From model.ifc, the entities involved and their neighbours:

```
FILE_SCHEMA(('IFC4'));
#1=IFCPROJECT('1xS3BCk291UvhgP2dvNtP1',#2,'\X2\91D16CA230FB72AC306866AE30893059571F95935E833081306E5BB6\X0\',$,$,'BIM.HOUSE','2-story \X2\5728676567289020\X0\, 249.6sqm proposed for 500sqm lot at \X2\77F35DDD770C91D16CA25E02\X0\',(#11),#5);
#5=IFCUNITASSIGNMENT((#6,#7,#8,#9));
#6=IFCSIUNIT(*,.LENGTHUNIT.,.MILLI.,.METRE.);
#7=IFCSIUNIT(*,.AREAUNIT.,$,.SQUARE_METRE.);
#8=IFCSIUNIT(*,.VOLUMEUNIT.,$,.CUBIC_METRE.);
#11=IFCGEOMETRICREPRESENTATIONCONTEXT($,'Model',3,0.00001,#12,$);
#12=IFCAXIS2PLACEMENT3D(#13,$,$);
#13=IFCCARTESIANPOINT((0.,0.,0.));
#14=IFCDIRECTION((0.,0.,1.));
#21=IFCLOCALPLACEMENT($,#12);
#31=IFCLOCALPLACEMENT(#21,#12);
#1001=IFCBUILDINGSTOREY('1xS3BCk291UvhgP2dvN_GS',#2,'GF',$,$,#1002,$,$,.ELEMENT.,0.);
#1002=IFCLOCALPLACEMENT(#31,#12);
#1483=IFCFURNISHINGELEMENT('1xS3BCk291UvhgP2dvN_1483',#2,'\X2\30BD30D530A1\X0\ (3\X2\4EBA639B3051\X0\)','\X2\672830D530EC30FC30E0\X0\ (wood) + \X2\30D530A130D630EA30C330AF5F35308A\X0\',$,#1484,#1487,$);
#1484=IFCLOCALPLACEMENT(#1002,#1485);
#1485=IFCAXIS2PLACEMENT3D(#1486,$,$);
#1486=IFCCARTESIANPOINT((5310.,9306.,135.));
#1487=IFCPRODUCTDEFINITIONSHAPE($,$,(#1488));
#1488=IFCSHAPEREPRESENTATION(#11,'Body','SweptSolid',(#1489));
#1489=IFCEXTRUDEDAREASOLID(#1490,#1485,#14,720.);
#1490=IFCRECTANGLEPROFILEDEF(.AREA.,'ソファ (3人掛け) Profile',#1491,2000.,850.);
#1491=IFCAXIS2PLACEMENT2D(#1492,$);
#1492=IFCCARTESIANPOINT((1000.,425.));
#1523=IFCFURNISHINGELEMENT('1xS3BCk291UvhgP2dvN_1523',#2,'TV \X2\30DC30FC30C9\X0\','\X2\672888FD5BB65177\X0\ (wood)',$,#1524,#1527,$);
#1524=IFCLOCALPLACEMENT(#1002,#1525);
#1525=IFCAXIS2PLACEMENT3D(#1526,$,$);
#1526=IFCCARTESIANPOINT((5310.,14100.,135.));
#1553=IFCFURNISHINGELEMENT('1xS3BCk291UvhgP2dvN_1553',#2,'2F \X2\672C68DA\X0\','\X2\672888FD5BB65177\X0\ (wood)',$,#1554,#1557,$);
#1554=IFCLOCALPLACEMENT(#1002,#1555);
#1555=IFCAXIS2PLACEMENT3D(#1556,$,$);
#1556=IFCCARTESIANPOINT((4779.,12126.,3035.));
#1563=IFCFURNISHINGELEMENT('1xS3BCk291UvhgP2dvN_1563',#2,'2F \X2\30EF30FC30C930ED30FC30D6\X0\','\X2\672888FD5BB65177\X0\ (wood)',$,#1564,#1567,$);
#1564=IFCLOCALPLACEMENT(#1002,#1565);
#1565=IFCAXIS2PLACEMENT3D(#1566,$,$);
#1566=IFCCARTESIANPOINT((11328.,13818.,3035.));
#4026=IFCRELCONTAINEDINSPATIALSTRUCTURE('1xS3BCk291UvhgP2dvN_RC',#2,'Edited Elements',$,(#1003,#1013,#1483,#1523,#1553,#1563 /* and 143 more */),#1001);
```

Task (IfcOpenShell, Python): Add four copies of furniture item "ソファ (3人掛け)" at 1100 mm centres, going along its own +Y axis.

```python
import ifcopenshell
import ifcopenshell.api.geometry
import ifcopenshell.api.root
import ifcopenshell.util.element
import ifcopenshell.util.placement
import ifcopenshell.util.unit

model = ifcopenshell.open("model.ifc")
unit_scale = ifcopenshell.util.unit.calculate_unit_scale(model)


def reuse_history(source, copy):
    """copy_class also copies each property set's owner history, people and application; keep the originals."""
    for rel in copy.IsDefinedBy:
        if rel.is_a("IfcRelDefinesByProperties") and (history := rel.RelatingPropertyDefinition.OwnerHistory):
            rel.RelatingPropertyDefinition.OwnerHistory = source.OwnerHistory
            ifcopenshell.util.element.remove_deep2(model, history)


source = model.by_guid("1xS3BCk291UvhgP2dvN_1483")
base = ifcopenshell.util.placement.get_local_placement(source.ObjectPlacement)
step = base[:3, 1] * 1.1 / unit_scale

for i in range(1, 5):
    copy = ifcopenshell.api.root.copy_class(model, product=source)
    copy.Representation = ifcopenshell.util.element.copy_deep(
        model, source.Representation, exclude=["IfcGeometricRepresentationContext", "IfcRepresentationMap"]
    )
    reuse_history(source, copy)
    matrix = base.copy()
    matrix[:3, 3] += i * step
    print("added at", matrix[:3, 3].round(3) + 0.0)
    ifcopenshell.api.geometry.edit_object_placement(model, product=copy, matrix=matrix, is_si=False)

model.write("model_rev.ifc")
```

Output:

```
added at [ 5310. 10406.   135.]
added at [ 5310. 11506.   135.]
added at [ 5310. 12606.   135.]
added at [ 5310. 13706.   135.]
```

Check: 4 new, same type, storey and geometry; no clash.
